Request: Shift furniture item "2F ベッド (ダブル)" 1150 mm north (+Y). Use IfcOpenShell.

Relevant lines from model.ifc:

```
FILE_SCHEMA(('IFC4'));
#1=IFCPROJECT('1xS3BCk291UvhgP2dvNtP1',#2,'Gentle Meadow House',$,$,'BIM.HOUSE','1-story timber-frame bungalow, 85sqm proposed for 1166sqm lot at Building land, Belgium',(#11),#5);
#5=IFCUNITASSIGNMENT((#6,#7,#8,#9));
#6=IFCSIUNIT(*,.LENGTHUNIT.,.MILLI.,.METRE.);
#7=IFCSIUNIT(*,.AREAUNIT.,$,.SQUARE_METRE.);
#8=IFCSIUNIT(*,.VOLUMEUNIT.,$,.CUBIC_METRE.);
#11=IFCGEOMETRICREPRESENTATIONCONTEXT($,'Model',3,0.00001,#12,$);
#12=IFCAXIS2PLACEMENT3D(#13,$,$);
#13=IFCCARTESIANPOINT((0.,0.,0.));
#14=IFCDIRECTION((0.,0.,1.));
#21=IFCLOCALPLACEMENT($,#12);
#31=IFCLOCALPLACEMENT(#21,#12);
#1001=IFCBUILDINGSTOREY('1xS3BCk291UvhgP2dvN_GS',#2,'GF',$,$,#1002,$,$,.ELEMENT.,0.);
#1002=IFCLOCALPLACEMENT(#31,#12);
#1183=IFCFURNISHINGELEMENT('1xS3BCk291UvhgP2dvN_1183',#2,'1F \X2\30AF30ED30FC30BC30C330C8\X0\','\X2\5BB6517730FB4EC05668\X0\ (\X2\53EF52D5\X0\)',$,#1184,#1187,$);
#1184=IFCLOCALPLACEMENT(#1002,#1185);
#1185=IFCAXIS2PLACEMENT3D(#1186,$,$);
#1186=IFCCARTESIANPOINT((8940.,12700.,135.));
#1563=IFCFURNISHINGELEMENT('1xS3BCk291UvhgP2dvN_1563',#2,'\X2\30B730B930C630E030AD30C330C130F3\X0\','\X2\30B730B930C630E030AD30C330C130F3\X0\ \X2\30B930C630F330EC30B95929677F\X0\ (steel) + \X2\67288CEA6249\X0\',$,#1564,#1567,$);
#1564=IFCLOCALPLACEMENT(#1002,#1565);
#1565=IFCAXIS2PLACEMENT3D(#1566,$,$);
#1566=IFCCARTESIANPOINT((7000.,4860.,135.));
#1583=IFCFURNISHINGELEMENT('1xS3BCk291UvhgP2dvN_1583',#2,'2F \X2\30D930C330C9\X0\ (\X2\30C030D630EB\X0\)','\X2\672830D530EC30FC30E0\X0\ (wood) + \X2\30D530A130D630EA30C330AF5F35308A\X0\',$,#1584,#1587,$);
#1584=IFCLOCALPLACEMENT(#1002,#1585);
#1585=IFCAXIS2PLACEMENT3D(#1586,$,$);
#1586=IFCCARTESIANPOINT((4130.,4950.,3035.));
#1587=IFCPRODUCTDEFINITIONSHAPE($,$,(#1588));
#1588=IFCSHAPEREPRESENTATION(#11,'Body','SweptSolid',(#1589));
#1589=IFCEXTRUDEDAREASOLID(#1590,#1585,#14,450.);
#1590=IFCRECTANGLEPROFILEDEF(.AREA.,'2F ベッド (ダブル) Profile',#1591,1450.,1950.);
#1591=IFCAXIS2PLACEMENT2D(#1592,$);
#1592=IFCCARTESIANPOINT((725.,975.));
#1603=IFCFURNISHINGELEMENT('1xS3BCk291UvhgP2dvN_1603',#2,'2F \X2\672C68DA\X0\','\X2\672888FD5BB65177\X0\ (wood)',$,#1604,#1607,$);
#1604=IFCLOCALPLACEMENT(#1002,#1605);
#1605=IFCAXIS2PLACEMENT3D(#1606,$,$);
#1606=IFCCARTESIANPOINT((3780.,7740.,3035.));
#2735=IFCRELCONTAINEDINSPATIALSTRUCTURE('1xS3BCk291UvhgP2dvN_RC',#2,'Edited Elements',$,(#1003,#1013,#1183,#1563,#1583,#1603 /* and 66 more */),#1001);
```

```python
import ifcopenshell
import ifcopenshell.api.geometry
import ifcopenshell.util.placement
import ifcopenshell.util.unit

model = ifcopenshell.open("model.ifc")
unit_scale = ifcopenshell.util.unit.calculate_unit_scale(model)

item = model.by_id(1583)
matrix = ifcopenshell.util.placement.get_local_placement(item.ObjectPlacement)
matrix[1, 3] += 1.15 / unit_scale
ifcopenshell.api.geometry.edit_object_placement(model, product=item, matrix=matrix, is_si=False)

print(ifcopenshell.util.placement.get_local_placement(item.ObjectPlacement).round(3) + 0.0)

model.write("model_rev.ifc")
```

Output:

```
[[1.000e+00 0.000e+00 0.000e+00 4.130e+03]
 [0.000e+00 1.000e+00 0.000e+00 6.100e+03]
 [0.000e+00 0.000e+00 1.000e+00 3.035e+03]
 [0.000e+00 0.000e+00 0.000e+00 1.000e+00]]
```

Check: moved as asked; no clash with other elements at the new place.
